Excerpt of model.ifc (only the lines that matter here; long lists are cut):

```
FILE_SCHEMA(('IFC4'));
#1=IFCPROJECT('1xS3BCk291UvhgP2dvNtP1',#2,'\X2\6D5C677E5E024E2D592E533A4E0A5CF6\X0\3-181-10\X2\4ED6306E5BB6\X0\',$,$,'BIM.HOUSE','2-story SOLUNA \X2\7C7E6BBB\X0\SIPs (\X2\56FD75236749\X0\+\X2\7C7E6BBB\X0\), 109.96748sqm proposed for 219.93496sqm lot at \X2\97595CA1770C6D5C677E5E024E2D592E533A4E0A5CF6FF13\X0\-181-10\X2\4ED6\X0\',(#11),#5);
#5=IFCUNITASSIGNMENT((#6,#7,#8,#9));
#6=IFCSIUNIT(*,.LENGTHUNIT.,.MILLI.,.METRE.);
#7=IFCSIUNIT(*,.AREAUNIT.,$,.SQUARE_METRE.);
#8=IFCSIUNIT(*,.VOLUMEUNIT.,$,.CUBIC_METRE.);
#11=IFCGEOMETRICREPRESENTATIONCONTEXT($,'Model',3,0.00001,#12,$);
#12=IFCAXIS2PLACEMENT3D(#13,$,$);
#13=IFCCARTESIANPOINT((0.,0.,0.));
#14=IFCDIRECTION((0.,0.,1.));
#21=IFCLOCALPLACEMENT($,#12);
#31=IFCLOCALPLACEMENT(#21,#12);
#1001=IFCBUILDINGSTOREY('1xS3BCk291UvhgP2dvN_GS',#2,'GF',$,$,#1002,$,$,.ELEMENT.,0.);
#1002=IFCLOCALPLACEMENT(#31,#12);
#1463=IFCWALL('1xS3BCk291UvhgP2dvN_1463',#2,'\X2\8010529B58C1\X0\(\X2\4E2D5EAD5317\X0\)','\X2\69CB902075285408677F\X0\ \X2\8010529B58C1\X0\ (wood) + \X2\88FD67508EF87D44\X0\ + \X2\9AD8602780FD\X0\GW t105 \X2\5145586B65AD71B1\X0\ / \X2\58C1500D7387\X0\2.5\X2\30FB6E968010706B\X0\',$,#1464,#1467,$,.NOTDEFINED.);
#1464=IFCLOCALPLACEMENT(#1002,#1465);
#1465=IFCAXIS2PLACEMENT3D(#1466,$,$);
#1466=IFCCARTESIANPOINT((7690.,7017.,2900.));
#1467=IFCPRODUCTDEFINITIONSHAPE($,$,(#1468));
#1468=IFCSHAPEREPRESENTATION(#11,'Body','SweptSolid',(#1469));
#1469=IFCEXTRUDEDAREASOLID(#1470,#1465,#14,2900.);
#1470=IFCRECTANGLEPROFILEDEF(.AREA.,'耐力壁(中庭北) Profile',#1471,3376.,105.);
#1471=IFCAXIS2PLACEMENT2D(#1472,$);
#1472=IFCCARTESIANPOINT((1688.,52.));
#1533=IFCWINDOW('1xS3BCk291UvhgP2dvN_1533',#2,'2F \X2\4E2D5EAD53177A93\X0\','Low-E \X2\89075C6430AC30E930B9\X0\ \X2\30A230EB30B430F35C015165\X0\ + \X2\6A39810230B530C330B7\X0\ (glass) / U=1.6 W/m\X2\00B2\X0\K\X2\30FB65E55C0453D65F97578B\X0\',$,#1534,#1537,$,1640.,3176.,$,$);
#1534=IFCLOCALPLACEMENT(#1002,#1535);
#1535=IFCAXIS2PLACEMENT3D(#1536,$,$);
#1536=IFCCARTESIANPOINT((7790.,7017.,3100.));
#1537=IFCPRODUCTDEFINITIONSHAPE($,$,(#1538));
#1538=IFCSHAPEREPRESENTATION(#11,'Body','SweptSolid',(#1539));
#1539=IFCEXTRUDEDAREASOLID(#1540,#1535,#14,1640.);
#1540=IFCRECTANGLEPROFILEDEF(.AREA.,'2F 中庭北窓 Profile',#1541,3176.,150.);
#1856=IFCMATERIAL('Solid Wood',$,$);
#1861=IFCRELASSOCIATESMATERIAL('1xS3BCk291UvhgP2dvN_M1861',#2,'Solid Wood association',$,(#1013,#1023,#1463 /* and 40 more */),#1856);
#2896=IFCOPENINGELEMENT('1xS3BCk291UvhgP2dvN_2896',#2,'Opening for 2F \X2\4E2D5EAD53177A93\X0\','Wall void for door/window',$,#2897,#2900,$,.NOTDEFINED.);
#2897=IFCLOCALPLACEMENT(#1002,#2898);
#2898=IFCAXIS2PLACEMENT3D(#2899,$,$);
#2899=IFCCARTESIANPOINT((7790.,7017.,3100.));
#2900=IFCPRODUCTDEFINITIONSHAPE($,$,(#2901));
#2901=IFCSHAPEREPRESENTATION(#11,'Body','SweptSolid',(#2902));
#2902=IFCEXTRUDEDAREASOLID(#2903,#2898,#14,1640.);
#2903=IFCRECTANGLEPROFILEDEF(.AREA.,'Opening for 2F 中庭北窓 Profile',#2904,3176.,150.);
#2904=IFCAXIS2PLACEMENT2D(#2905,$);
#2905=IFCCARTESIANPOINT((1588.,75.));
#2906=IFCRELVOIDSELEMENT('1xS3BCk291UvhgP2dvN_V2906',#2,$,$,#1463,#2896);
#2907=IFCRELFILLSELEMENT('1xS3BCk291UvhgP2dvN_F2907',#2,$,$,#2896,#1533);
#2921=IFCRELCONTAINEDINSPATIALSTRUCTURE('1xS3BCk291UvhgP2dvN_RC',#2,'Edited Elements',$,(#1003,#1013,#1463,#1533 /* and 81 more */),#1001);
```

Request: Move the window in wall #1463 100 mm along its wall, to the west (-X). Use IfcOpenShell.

```python
import ifcopenshell
import ifcopenshell.api.geometry
import ifcopenshell.util.placement
import ifcopenshell.util.unit

model = ifcopenshell.open("model.ifc")
unit_scale = ifcopenshell.util.unit.calculate_unit_scale(model)

window = model.by_guid("1xS3BCk291UvhgP2dvN_1533")
opening = window.FillsVoids[0].RelatingOpeningElement
wall = opening.VoidsElements[0].RelatingBuildingElement

wall_matrix = ifcopenshell.util.placement.get_local_placement(wall.ObjectPlacement)
shift = wall_matrix[:3, 0] * -0.1 / unit_scale
before = ifcopenshell.util.placement.get_local_placement(window.ObjectPlacement)[:3, 3].copy()

# The window is not placed relative to its opening, so move both.
for product in (opening, window):
    matrix = ifcopenshell.util.placement.get_local_placement(product.ObjectPlacement)
    matrix[:3, 3] += shift
    ifcopenshell.api.geometry.edit_object_placement(model, product=product, matrix=matrix, is_si=False)

after = ifcopenshell.util.placement.get_local_placement(window.ObjectPlacement)[:3, 3]
print("window moved by", (after - before).round(3) + 0.0)

model.write("model_rev.ifc")
```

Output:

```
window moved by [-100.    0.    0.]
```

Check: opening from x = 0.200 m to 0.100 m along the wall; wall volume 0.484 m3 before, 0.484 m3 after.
